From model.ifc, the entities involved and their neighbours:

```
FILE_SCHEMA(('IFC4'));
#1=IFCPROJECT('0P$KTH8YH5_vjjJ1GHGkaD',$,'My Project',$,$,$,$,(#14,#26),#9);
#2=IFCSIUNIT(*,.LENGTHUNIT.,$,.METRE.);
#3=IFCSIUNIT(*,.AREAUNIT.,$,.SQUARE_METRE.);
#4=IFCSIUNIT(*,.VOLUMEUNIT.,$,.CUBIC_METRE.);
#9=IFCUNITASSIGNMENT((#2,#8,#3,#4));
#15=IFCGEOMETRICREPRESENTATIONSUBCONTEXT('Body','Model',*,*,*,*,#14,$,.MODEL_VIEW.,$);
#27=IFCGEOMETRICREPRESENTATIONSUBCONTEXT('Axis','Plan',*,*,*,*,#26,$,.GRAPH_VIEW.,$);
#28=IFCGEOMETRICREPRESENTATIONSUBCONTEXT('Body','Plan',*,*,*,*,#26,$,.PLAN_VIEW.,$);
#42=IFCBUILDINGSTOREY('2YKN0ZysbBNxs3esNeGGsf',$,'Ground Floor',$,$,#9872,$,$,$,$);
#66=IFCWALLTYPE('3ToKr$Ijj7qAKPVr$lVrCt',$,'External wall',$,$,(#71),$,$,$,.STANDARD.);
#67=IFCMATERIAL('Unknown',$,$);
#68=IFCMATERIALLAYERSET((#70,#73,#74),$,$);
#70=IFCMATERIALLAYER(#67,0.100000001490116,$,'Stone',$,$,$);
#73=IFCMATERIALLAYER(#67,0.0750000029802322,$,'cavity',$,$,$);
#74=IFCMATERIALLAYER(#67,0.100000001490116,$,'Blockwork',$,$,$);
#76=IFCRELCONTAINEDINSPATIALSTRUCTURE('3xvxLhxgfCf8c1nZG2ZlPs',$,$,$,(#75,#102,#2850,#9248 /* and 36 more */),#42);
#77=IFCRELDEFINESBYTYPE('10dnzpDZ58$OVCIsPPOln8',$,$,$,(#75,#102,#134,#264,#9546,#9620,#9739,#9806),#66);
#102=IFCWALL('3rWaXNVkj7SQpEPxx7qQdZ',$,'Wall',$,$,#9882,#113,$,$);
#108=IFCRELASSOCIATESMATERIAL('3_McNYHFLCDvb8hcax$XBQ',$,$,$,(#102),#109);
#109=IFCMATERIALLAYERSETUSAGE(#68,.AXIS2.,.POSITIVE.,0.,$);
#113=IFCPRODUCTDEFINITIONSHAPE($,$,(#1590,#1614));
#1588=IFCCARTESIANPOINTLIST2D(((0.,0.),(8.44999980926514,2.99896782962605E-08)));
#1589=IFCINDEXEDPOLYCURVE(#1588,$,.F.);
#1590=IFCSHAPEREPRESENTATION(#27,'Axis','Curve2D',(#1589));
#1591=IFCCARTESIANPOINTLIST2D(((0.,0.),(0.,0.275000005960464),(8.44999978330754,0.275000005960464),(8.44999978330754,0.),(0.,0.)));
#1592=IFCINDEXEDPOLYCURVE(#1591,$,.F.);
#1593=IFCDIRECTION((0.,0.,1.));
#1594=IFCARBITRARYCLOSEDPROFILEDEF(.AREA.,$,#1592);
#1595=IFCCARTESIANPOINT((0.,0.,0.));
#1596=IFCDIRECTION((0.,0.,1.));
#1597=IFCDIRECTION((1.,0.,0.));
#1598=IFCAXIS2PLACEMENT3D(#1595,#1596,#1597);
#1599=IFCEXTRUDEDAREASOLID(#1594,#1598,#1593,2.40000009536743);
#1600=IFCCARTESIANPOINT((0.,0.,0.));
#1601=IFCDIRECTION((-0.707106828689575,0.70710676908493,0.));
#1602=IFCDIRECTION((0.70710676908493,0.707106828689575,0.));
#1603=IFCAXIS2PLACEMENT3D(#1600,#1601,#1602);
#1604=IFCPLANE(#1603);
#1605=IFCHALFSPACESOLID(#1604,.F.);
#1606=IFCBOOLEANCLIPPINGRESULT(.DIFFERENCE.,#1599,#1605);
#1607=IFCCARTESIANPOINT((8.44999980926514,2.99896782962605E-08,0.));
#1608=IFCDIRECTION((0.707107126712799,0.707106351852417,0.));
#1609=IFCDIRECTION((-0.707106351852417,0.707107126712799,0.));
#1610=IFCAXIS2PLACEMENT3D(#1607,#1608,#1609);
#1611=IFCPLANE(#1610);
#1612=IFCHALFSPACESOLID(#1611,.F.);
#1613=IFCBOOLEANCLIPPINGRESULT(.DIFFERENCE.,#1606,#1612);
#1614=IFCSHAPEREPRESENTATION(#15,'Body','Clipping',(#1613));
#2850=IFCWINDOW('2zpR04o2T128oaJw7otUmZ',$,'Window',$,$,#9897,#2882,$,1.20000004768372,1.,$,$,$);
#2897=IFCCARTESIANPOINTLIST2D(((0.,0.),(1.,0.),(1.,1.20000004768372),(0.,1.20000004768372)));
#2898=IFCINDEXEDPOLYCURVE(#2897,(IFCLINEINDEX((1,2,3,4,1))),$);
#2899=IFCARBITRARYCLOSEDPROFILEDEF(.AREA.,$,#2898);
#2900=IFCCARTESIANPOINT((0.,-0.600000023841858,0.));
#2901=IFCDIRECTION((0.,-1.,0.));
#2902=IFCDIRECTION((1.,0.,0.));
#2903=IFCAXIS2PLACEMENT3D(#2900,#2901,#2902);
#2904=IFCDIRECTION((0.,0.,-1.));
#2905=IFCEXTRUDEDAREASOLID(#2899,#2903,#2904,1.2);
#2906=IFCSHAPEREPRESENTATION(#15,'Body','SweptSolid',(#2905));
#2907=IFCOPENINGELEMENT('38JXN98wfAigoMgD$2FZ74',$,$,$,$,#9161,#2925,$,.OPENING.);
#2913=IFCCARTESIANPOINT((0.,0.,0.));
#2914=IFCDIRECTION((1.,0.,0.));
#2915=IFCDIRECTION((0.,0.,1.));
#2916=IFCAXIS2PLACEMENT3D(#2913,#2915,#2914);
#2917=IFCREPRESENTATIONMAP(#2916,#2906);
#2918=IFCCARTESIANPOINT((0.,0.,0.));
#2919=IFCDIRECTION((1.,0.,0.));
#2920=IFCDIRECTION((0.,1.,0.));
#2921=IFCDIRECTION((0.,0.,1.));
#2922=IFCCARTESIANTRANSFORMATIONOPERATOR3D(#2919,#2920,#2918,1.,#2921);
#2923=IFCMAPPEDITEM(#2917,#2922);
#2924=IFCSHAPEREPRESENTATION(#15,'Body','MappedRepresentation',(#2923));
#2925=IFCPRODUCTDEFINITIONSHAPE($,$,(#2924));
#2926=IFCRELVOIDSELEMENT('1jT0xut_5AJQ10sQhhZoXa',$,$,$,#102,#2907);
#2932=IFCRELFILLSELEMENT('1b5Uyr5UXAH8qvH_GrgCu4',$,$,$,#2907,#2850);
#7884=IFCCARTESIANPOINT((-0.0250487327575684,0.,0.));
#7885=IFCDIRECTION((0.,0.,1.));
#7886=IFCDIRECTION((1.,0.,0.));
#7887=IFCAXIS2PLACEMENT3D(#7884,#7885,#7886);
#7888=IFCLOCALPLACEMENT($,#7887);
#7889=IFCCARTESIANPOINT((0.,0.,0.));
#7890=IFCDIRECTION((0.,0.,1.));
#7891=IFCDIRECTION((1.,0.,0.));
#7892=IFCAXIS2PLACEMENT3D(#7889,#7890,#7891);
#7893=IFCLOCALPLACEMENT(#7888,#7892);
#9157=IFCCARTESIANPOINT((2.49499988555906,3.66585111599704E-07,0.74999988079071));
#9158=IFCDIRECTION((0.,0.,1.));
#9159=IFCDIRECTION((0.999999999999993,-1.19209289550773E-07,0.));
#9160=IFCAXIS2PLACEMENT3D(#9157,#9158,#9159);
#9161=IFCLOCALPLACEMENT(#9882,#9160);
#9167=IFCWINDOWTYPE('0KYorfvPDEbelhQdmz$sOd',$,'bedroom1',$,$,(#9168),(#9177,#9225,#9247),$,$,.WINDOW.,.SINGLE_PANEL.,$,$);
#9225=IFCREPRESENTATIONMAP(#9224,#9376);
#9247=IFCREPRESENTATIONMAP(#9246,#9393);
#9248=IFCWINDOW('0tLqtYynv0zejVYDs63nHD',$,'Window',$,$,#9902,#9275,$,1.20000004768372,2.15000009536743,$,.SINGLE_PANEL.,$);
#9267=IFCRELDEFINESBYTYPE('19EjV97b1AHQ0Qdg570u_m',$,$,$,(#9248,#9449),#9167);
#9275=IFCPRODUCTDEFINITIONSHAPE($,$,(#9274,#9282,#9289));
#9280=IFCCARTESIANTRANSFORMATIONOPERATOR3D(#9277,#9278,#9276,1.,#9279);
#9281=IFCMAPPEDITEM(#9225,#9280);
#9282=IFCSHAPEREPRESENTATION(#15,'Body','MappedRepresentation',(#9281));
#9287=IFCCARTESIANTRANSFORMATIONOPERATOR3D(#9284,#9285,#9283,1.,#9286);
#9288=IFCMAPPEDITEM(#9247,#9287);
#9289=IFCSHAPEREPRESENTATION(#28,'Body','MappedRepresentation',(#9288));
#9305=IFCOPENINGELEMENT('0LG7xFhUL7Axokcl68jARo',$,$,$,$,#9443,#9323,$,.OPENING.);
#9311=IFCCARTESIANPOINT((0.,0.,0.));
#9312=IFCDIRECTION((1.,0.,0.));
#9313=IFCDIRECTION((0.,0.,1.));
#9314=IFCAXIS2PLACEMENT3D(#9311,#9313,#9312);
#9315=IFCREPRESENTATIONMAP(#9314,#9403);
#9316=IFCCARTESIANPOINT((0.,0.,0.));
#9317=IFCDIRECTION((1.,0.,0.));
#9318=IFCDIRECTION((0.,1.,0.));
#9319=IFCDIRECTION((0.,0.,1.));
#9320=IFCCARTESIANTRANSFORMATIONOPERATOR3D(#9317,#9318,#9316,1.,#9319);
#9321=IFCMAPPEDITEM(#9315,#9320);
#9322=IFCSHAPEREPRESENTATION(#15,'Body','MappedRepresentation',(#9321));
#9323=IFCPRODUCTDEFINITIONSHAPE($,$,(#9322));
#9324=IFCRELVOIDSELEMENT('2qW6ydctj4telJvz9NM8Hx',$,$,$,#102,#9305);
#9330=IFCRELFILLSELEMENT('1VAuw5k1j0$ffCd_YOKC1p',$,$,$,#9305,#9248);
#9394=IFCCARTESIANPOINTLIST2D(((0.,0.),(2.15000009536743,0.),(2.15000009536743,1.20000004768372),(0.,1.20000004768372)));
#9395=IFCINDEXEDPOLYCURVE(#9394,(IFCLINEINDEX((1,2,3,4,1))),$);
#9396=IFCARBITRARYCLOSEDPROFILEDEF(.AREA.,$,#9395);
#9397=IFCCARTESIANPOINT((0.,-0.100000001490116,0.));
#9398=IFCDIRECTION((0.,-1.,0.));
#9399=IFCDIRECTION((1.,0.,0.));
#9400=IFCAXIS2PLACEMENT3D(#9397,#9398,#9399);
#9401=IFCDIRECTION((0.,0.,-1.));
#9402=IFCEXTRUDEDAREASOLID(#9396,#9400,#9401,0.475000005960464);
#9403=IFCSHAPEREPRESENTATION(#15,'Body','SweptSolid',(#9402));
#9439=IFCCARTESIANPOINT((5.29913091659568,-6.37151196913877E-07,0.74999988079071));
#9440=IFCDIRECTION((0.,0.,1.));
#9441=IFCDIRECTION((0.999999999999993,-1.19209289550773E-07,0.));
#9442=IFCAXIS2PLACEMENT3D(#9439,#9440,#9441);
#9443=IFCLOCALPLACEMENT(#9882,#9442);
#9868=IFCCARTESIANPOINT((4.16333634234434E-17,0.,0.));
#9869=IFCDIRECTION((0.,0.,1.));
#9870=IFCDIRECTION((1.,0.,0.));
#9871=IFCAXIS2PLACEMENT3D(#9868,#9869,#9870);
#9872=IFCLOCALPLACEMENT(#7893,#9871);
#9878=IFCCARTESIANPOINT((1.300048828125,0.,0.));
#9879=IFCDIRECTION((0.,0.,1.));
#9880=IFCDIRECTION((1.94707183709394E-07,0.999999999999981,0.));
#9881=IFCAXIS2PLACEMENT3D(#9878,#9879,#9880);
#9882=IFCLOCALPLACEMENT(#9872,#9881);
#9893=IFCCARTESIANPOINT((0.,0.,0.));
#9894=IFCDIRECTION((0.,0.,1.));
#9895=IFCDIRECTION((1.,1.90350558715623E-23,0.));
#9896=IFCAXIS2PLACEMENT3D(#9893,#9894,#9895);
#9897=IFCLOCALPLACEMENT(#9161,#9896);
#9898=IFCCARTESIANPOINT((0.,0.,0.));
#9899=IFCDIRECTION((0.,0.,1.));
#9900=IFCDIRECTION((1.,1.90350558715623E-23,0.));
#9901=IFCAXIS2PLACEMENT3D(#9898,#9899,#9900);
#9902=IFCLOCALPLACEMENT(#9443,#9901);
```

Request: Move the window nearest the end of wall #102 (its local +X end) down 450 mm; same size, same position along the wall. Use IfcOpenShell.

```python
import numpy as np
import ifcopenshell
import ifcopenshell.api.geometry
import ifcopenshell.util.placement
import ifcopenshell.util.unit

model = ifcopenshell.open("model.ifc")
unit_scale = ifcopenshell.util.unit.calculate_unit_scale(model)

window = model.by_id(9248)
opening = window.FillsVoids[0].RelatingOpeningElement
dz = -0.45

shift = np.array([0.0, 0.0, dz])
# The window is placed relative to its opening, so it follows when the opening moves.
matrix = ifcopenshell.util.placement.get_local_placement(opening.ObjectPlacement)
matrix[:3, 3] += shift
ifcopenshell.api.geometry.edit_object_placement(
    model, product=opening, matrix=matrix, is_si=False, should_transform_children=True
)

print(f"moved by {dz * unit_scale:+.3f} m")

model.write("model-out.ifc")
```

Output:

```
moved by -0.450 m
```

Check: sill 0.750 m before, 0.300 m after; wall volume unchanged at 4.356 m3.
